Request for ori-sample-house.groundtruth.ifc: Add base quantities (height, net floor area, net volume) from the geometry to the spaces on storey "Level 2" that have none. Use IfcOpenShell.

First a look at what the model holds.

```python
import ifcopenshell
import ifcopenshell.util.element
import ifcopenshell.util.unit

model = ifcopenshell.open("ori-sample-house.groundtruth.ifc")
print(model.schema)
for unit_type in ("LENGTHUNIT", "AREAUNIT", "VOLUMEUNIT"):
    print(unit_type, ifcopenshell.util.unit.calculate_unit_scale(model, unit_type))
storey = next(s for s in model.by_type("IfcBuildingStorey") if s.Name == "Level 2")
spaces = [e for e in ifcopenshell.util.element.get_decomposition(storey) if e.is_a("IfcSpace")]
for e in sorted(spaces, key=lambda e: e.id()):
    print(e.id(), e.is_a(), e.Name, list(ifcopenshell.util.element.get_psets(e, qtos_only=True)), sep=" | ")
```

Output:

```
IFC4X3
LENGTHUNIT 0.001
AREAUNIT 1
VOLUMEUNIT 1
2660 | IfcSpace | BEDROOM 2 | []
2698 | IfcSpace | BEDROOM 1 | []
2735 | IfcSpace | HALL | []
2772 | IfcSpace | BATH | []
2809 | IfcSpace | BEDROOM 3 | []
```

```python
import ifcopenshell
import ifcopenshell.api.pset
import ifcopenshell.geom
import ifcopenshell.util.element
import ifcopenshell.util.shape
import ifcopenshell.util.unit

model = ifcopenshell.open("ori-sample-house.groundtruth.ifc")
unit_scale = ifcopenshell.util.unit.calculate_unit_scale(model)
area_scale = ifcopenshell.util.unit.calculate_unit_scale(model, "AREAUNIT")
volume_scale = ifcopenshell.util.unit.calculate_unit_scale(model, "VOLUMEUNIT")
settings = ifcopenshell.geom.settings()

storey = next(s for s in model.by_type("IfcBuildingStorey") if s.Name == "Level 2")
spaces = [e for e in ifcopenshell.util.element.get_decomposition(storey) if e.is_a("IfcSpace")]

for e in sorted(spaces, key=lambda e: e.id()):
    if ifcopenshell.util.element.get_psets(e, qtos_only=True, should_inherit=False):
        continue
    # Geometry comes back in metres, in the element's own axes.
    shape = ifcopenshell.geom.create_shape(settings, e)
    values = {
        "Height": ifcopenshell.util.shape.get_z(shape.geometry) / unit_scale,
        "NetFloorArea": ifcopenshell.util.shape.get_footprint_area(shape.geometry) / area_scale,
        "NetVolume": ifcopenshell.util.shape.get_volume(shape.geometry) / volume_scale,
    }
    qto = ifcopenshell.api.pset.add_qto(model, product=e, name="Qto_SpaceBaseQuantities")
    ifcopenshell.api.pset.edit_qto(model, qto=qto, properties=values)
    print(e.id(), {k: round(v, 3) for k, v in values.items()})

model.write("ori-sample-house.groundtruth_updated.ifc")
```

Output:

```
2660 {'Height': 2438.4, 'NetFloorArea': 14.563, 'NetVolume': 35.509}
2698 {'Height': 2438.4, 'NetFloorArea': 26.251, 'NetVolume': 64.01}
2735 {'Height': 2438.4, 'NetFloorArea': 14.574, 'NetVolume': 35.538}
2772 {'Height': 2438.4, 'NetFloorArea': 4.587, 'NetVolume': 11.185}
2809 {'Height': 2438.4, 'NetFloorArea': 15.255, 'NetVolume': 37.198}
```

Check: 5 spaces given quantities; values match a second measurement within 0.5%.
